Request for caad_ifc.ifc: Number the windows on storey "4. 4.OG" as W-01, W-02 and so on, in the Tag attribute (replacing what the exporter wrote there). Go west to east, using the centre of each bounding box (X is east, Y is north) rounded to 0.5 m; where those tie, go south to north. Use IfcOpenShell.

First a look at what the model holds.

```python
import ifcopenshell
import ifcopenshell.util.element
import ifcopenshell.util.placement

model = ifcopenshell.open("caad_ifc.ifc")
print(model.schema)
storey = next(s for s in model.by_type("IfcBuildingStorey") if s.Name == "4. 4.OG")
windows = [e for e in ifcopenshell.util.element.get_decomposition(storey) if e.is_a("IfcWindow")]
for e in sorted(windows, key=lambda e: e.id()):
    origin = ifcopenshell.util.placement.get_local_placement(e.ObjectPlacement)[:3, 3]
    print(e.id(), e.Tag, e.Name, origin.round(2) + 0.0, sep=" | ")
```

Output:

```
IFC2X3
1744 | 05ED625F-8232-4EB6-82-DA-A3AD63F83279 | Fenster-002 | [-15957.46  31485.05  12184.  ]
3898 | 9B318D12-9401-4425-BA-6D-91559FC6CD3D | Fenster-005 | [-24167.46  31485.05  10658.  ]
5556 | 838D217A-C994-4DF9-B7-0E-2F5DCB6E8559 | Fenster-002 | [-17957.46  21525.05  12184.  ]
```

```python
import ifcopenshell
import ifcopenshell.geom
import ifcopenshell.util.element
import ifcopenshell.util.shape

model = ifcopenshell.open("caad_ifc.ifc")
settings = ifcopenshell.geom.settings()
settings.set("use-world-coords", True)


def centre(element):
    shape = ifcopenshell.geom.create_shape(settings, element)
    return ifcopenshell.util.shape.get_bbox_centroid(shape.geometry)


storey = next(s for s in model.by_type("IfcBuildingStorey") if s.Name == "4. 4.OG")
windows = [e for e in ifcopenshell.util.element.get_decomposition(storey) if e.is_a("IfcWindow")]

# Insertion points can sit at a corner or the storey origin, so sort by the geometry (in metres).
centres = {e: centre(e) for e in windows}
windows.sort(key=lambda e: (round(centres[e][0] / 0.5), centres[e][1]))

for i, e in enumerate(windows, start=1):
    number = f"W-{i:02d}"
    e.Tag = number
    print(e.id(), number)

model.write("caad_ifc_v2.ifc")
```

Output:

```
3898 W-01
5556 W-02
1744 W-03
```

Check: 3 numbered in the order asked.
